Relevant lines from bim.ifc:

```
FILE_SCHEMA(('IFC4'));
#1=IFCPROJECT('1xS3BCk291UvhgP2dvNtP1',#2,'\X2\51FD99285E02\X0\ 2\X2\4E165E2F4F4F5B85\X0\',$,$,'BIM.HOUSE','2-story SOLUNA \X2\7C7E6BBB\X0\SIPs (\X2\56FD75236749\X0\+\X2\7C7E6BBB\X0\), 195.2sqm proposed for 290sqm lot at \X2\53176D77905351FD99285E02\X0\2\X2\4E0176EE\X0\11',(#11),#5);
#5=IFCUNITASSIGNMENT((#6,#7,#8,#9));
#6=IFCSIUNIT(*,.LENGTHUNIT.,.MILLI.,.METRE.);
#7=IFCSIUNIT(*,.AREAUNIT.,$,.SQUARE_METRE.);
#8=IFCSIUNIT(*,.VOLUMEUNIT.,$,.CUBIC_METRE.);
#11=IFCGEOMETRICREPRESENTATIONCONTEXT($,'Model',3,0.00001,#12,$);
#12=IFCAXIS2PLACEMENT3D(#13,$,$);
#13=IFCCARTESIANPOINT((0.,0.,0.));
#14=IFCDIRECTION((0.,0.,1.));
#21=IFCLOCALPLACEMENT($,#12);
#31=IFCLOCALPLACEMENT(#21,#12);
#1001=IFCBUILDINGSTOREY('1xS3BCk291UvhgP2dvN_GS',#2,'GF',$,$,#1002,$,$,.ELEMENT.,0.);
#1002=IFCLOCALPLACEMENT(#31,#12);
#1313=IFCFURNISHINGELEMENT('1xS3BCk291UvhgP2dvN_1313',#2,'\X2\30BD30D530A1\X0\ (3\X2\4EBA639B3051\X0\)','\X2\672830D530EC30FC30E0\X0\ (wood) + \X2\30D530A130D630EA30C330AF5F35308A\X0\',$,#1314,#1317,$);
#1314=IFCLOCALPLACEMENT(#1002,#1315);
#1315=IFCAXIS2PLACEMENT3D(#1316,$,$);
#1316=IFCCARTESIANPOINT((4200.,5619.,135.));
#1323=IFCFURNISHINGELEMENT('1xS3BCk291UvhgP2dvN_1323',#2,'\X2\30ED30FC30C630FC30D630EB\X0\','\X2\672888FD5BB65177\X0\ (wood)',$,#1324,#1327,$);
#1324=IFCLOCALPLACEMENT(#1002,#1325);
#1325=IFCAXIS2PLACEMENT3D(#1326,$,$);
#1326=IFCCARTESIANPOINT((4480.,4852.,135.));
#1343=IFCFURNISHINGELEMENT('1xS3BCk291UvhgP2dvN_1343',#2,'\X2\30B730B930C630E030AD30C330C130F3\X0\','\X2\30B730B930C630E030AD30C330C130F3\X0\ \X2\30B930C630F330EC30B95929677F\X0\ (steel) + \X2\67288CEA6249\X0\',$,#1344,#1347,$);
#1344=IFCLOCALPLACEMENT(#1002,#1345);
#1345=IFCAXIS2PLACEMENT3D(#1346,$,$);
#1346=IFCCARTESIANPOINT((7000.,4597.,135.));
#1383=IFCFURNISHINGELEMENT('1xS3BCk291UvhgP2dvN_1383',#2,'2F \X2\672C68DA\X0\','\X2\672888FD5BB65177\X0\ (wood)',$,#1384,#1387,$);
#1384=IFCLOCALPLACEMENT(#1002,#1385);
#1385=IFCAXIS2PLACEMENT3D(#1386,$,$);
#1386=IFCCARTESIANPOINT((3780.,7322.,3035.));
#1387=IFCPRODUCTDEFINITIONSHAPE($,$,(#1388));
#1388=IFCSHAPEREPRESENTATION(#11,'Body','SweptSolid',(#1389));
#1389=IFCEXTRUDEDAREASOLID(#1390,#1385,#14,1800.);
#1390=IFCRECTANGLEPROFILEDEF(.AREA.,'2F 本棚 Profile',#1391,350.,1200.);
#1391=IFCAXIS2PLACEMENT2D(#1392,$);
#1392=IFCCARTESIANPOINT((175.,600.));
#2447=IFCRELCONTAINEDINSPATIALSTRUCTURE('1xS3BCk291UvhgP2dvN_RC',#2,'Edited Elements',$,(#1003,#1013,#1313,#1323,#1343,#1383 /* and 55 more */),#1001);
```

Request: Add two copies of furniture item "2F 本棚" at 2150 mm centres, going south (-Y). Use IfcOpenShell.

```python
import numpy as np
import ifcopenshell
import ifcopenshell.api.geometry
import ifcopenshell.api.root
import ifcopenshell.util.element
import ifcopenshell.util.placement
import ifcopenshell.util.unit

model = ifcopenshell.open("bim.ifc")
unit_scale = ifcopenshell.util.unit.calculate_unit_scale(model)


def reuse_history(source, copy):
    """copy_class also copies each property set's owner history, people and application; keep the originals."""
    for rel in copy.IsDefinedBy:
        if rel.is_a("IfcRelDefinesByProperties") and (history := rel.RelatingPropertyDefinition.OwnerHistory):
            rel.RelatingPropertyDefinition.OwnerHistory = source.OwnerHistory
            ifcopenshell.util.element.remove_deep2(model, history)


source = model.by_guid("1xS3BCk291UvhgP2dvN_1383")
base = ifcopenshell.util.placement.get_local_placement(source.ObjectPlacement)
step = np.array([0.0, -1.0, 0.0]) * 2.15 / unit_scale

for i in range(1, 3):
    copy = ifcopenshell.api.root.copy_class(model, product=source)
    copy.Representation = ifcopenshell.util.element.copy_deep(
        model, source.Representation, exclude=["IfcGeometricRepresentationContext", "IfcRepresentationMap"]
    )
    reuse_history(source, copy)
    matrix = base.copy()
    matrix[:3, 3] += i * step
    print("added at", matrix[:3, 3].round(3) + 0.0)
    ifcopenshell.api.geometry.edit_object_placement(model, product=copy, matrix=matrix, is_si=False)

model.write("bim-out.ifc")
```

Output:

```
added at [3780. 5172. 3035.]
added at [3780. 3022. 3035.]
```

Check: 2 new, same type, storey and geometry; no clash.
